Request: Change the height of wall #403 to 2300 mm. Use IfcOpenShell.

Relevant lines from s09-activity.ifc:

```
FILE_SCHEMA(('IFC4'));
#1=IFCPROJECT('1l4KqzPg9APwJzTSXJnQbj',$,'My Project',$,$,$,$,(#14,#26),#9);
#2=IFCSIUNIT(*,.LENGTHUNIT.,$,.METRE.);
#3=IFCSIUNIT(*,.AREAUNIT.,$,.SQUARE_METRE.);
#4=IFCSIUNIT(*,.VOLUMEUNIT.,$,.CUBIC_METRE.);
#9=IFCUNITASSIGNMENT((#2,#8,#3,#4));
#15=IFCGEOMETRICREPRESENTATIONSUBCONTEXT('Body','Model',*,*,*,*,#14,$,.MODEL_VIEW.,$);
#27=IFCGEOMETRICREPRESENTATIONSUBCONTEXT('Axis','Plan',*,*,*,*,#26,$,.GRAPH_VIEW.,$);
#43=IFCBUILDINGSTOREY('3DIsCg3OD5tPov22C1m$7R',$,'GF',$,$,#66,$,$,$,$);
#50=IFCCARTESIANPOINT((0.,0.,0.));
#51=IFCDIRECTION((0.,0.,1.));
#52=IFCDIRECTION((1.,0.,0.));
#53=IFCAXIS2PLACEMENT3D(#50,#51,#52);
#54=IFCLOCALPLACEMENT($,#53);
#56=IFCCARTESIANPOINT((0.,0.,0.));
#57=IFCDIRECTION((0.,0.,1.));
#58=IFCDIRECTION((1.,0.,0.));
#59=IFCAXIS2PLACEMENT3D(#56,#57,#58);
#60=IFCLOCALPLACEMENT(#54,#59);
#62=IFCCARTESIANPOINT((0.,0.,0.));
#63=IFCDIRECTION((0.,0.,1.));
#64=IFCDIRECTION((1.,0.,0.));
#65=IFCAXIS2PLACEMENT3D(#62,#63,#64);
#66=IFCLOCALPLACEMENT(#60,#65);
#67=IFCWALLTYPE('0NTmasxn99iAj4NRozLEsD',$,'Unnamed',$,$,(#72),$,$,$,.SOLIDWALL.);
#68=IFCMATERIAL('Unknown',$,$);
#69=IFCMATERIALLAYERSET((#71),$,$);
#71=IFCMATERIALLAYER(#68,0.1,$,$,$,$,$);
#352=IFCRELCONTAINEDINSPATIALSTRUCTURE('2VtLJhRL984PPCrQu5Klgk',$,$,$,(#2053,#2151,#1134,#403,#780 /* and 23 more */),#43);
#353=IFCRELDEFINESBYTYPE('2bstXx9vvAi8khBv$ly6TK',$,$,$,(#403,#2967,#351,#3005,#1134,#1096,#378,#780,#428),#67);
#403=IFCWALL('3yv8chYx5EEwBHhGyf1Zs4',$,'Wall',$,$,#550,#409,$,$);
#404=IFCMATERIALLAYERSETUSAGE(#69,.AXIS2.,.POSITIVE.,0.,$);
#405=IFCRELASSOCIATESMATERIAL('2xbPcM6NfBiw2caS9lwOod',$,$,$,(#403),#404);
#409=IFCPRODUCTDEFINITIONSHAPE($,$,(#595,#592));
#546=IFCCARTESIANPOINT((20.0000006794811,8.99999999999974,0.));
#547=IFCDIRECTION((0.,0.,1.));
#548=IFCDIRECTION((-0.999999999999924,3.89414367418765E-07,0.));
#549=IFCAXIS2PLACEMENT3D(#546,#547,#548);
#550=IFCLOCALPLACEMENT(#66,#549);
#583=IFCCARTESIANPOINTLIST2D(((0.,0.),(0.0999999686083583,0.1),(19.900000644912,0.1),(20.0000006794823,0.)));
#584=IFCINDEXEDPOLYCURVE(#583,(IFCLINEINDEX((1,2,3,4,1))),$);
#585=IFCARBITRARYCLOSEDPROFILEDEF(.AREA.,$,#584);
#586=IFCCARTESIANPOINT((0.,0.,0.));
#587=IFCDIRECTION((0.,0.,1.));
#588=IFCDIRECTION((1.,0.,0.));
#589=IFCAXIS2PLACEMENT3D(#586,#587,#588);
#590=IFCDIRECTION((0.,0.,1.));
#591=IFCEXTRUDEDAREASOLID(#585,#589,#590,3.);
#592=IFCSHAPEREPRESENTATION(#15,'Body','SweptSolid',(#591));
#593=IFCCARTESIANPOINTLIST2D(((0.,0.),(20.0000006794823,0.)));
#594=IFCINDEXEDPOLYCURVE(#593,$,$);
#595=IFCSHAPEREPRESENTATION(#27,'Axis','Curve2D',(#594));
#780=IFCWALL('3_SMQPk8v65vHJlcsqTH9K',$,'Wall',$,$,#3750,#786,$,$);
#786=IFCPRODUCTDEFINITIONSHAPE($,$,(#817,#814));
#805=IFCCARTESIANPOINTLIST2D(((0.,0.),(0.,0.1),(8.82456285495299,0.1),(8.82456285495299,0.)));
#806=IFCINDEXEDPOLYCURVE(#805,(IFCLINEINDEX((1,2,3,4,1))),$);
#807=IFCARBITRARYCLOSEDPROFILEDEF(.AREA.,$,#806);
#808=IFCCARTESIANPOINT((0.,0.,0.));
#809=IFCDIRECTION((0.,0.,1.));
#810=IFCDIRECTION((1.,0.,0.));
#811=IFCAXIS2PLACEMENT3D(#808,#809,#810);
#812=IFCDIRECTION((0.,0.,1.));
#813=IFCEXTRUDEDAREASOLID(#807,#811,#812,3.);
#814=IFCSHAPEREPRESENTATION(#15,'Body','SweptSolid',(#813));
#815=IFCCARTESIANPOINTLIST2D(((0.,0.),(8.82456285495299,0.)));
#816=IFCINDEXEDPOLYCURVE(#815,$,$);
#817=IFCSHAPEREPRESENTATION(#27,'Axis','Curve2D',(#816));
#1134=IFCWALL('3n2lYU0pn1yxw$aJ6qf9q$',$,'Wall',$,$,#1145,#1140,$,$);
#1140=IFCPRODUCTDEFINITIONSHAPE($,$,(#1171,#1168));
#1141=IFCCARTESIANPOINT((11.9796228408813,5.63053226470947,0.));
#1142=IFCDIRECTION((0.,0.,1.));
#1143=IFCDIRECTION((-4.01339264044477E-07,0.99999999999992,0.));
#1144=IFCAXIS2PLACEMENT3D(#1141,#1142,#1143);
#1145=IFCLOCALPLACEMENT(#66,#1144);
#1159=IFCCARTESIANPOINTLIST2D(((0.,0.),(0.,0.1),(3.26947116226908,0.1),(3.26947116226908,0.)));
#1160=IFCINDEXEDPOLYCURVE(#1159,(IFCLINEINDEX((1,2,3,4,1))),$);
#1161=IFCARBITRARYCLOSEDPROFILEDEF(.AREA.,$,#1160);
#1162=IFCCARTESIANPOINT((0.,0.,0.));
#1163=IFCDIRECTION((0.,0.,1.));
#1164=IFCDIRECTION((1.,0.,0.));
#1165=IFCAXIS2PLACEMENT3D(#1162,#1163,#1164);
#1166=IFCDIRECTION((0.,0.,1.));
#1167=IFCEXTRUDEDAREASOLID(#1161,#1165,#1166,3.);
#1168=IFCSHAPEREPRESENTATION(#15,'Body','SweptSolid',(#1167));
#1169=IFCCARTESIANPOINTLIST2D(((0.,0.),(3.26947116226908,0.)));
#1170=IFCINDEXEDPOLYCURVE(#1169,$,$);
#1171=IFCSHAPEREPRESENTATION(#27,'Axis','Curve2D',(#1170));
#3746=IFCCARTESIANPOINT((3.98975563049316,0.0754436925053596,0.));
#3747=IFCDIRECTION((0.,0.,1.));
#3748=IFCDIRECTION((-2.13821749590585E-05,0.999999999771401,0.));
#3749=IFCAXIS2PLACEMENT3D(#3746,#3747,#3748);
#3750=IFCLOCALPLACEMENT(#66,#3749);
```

```python
import ifcopenshell
import ifcopenshell.geom
import ifcopenshell.util.representation
import ifcopenshell.util.shape

model = ifcopenshell.open("s09-activity.ifc")
settings = ifcopenshell.geom.settings()


def volume(element):
    """Net volume in cubic metres, openings subtracted."""
    shape = ifcopenshell.geom.create_shape(settings, element)
    return ifcopenshell.util.shape.get_volume(shape.geometry)


wall = model.by_guid("3yv8chYx5EEwBHhGyf1Zs4")
before = volume(wall)

body = ifcopenshell.util.representation.get_representation(wall, "Model", "Body")
solid = body.Items[0]
old_height = solid.Depth
solid.Depth = 2.3
after = volume(wall)

print(f"height {old_height:g} -> {solid.Depth:g}, volume {before:.3f} -> {after:.3f} m3")

model.write("s09-activity_updated.ifc")
```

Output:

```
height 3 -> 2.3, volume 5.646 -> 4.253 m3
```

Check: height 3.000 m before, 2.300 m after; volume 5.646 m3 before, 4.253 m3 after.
